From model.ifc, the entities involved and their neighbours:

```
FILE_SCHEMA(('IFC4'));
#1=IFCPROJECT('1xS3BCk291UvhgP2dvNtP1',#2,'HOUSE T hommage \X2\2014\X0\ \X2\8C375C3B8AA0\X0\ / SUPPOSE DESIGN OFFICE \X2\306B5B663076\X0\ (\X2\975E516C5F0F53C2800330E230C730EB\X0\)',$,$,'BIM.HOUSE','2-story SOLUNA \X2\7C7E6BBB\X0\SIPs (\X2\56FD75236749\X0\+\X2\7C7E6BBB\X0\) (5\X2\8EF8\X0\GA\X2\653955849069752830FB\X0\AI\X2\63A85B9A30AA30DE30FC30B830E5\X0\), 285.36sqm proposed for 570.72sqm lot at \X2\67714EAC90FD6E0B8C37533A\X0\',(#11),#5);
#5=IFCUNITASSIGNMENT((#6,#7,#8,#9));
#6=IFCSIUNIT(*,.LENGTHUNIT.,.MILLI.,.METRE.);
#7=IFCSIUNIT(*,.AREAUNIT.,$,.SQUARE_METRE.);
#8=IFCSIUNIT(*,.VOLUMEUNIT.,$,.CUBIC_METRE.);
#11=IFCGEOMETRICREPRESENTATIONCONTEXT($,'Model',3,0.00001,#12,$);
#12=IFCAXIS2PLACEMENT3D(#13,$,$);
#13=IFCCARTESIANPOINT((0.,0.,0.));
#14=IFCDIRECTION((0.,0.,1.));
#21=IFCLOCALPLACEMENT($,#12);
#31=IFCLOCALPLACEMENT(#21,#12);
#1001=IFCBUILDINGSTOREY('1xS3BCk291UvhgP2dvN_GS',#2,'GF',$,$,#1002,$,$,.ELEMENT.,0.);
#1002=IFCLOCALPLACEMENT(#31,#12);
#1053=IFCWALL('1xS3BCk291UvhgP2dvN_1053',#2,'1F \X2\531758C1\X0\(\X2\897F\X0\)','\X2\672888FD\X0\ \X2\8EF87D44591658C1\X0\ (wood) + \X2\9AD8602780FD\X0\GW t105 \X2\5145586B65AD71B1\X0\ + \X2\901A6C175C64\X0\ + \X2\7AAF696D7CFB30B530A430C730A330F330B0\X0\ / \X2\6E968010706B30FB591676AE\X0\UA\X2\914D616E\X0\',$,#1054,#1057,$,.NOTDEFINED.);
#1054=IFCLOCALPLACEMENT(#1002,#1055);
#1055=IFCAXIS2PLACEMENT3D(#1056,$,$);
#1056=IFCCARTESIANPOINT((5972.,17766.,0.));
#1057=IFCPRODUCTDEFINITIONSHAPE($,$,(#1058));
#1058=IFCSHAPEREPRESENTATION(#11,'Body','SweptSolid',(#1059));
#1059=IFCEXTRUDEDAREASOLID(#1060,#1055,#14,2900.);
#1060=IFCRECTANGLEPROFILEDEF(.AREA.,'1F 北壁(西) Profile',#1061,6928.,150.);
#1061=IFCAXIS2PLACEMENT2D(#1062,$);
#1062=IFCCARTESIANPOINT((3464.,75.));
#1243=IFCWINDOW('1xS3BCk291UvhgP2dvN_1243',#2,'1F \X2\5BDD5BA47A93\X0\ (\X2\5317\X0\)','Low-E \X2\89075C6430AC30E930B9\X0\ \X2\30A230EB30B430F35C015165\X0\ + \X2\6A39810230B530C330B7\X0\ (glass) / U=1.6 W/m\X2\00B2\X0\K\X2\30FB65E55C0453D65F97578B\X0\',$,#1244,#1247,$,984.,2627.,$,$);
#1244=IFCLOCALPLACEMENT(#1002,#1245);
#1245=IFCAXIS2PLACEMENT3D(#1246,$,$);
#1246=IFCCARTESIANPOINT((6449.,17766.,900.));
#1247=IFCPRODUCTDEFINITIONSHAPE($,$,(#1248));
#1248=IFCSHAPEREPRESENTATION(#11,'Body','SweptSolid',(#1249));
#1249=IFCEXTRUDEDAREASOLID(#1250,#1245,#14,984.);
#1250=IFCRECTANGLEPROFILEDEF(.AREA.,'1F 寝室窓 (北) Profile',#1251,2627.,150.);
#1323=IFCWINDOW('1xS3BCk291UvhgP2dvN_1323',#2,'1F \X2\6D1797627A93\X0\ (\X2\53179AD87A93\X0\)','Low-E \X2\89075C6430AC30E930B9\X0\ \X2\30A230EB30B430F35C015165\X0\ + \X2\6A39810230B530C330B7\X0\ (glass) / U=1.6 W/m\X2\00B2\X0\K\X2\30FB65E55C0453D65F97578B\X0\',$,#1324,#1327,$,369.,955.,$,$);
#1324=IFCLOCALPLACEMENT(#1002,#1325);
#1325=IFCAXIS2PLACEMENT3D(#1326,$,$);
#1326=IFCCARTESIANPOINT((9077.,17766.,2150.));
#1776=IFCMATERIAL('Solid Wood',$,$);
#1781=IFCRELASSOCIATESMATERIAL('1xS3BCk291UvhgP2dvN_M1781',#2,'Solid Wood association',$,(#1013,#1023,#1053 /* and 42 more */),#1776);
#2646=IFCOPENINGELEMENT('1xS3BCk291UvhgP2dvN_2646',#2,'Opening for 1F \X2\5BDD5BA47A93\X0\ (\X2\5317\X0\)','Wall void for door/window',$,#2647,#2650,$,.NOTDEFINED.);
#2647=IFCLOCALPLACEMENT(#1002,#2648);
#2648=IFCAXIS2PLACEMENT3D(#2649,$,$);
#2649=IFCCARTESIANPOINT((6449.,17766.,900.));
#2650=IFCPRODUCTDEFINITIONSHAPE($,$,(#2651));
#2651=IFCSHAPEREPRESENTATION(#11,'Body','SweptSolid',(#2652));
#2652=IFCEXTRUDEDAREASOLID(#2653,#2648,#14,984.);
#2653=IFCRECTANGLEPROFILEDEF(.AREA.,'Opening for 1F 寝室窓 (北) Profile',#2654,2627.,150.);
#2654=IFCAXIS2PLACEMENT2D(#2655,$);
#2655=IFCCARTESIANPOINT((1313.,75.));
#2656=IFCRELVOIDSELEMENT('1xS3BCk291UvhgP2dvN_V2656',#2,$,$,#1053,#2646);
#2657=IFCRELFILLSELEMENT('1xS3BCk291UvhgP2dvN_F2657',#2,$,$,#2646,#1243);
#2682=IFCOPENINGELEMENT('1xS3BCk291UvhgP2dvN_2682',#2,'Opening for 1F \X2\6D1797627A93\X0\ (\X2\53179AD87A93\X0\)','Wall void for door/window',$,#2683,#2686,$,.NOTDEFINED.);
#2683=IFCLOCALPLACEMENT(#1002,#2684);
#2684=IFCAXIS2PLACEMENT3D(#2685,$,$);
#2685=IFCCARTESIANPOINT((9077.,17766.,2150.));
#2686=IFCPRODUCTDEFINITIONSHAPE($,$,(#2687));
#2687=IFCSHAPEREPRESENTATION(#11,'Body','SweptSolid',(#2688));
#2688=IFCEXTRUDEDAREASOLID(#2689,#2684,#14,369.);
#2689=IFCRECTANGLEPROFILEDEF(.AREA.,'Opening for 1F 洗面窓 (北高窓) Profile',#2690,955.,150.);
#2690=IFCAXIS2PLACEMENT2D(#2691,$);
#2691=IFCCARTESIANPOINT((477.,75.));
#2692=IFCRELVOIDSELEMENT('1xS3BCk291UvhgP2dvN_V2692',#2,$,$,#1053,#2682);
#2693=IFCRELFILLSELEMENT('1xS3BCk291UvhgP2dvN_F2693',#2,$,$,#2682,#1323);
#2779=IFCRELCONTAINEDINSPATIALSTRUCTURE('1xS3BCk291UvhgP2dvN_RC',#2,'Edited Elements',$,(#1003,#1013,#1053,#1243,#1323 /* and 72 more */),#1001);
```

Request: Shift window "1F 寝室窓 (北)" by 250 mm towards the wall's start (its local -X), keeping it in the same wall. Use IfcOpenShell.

```python
import ifcopenshell
import ifcopenshell.api.geometry
import ifcopenshell.util.placement

model = ifcopenshell.open("model.ifc")

window = model.by_guid("1xS3BCk291UvhgP2dvN_1243")
opening = window.FillsVoids[0].RelatingOpeningElement
wall = opening.VoidsElements[0].RelatingBuildingElement

wall_matrix = ifcopenshell.util.placement.get_local_placement(wall.ObjectPlacement)
shift = wall_matrix[:3, 0] * -250.0
before = ifcopenshell.util.placement.get_local_placement(window.ObjectPlacement)[:3, 3].copy()

# The window is not placed relative to its opening, so move both.
for product in (opening, window):
    matrix = ifcopenshell.util.placement.get_local_placement(product.ObjectPlacement)
    matrix[:3, 3] += shift
    ifcopenshell.api.geometry.edit_object_placement(model, product=product, matrix=matrix, is_si=False)

after = ifcopenshell.util.placement.get_local_placement(window.ObjectPlacement)[:3, 3]
print("window moved by", (after - before).round(3) + 0.0)

model.write("model_v2.ifc")
```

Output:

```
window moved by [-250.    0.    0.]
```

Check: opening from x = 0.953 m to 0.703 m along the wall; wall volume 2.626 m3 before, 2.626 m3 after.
